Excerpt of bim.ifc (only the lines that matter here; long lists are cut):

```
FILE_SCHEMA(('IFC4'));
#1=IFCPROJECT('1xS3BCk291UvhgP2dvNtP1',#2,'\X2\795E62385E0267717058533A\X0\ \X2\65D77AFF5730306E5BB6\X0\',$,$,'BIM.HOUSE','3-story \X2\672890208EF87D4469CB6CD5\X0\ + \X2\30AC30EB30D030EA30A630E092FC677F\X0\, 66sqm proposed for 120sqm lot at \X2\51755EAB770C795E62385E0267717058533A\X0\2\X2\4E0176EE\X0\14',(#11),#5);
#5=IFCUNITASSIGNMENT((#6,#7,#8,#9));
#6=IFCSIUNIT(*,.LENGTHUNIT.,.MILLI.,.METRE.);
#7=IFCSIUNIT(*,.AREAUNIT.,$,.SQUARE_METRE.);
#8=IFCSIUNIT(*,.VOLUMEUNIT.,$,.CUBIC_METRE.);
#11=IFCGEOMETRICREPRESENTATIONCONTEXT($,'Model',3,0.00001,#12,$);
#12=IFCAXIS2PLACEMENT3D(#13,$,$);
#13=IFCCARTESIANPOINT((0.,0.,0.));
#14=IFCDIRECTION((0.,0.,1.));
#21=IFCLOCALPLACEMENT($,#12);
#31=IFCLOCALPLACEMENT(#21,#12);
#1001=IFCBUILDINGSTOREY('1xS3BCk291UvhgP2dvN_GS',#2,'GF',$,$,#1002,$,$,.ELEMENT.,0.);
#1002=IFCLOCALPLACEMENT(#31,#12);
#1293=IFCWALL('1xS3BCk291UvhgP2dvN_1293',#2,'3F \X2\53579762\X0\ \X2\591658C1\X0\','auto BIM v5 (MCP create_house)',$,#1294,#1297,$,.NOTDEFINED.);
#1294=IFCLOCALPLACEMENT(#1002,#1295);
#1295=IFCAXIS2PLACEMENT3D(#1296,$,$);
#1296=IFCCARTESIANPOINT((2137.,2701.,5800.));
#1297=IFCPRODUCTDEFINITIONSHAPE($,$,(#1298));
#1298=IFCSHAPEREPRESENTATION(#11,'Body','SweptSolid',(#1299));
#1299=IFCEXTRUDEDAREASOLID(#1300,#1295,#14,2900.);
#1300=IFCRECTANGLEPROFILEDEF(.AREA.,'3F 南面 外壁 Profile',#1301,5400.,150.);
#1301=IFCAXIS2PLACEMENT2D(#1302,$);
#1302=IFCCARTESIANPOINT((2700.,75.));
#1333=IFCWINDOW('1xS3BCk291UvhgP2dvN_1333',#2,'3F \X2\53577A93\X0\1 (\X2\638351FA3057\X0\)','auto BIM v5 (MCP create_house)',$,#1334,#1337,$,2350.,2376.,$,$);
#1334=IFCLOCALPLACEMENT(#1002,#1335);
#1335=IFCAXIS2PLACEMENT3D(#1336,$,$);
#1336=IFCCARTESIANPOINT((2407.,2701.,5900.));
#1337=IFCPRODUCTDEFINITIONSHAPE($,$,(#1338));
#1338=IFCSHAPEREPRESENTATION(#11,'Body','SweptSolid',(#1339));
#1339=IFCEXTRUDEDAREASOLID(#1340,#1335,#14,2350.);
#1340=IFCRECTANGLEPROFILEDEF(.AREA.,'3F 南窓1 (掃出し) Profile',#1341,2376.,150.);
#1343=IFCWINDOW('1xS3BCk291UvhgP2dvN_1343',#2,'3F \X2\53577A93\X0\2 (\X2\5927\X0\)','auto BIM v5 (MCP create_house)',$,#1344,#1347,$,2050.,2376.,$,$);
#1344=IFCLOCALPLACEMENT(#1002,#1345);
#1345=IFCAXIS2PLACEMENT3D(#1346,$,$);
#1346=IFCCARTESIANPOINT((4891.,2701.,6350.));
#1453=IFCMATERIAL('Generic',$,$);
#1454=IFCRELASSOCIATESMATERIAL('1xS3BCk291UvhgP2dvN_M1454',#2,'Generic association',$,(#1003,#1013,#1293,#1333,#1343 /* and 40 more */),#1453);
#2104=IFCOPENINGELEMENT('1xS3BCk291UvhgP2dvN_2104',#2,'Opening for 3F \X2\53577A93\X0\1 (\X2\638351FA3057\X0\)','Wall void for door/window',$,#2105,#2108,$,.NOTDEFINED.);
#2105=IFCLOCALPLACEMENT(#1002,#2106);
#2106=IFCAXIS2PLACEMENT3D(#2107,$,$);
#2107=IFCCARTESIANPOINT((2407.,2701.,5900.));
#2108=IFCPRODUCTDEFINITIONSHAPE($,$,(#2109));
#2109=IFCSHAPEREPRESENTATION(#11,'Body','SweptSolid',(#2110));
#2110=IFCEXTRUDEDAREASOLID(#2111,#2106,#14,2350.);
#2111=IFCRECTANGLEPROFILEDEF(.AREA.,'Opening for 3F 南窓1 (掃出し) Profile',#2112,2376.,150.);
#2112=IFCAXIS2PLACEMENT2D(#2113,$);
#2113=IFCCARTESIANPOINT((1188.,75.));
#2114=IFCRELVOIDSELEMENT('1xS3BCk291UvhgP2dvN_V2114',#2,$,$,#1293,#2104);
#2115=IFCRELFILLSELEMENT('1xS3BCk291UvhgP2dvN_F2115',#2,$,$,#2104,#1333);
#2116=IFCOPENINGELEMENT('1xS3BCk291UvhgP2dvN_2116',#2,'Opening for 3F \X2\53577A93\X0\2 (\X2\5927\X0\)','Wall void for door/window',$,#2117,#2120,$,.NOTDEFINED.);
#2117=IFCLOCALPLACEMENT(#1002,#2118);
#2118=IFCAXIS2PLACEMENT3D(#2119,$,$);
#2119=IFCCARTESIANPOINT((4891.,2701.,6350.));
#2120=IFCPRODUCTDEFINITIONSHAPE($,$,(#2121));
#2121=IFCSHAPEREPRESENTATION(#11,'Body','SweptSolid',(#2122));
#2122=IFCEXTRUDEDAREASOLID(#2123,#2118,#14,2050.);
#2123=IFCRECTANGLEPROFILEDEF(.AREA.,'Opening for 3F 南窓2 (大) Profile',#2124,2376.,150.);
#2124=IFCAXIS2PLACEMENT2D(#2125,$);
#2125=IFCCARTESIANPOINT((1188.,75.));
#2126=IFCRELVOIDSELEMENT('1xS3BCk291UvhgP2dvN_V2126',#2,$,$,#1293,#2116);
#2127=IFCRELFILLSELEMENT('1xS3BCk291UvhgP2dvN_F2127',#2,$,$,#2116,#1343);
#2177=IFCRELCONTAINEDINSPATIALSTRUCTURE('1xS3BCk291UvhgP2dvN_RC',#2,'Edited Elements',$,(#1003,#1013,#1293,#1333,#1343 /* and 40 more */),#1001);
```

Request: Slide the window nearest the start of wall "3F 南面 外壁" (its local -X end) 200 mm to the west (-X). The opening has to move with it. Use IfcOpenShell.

```python
import ifcopenshell
import ifcopenshell.api.geometry
import ifcopenshell.util.placement

model = ifcopenshell.open("bim.ifc")

window = model.by_id(1333)
opening = window.FillsVoids[0].RelatingOpeningElement
wall = opening.VoidsElements[0].RelatingBuildingElement

wall_matrix = ifcopenshell.util.placement.get_local_placement(wall.ObjectPlacement)
shift = wall_matrix[:3, 0] * -200.0
before = ifcopenshell.util.placement.get_local_placement(window.ObjectPlacement)[:3, 3].copy()

# The window is not placed relative to its opening, so move both.
for product in (opening, window):
    matrix = ifcopenshell.util.placement.get_local_placement(product.ObjectPlacement)
    matrix[:3, 3] += shift
    ifcopenshell.api.geometry.edit_object_placement(model, product=product, matrix=matrix, is_si=False)

after = ifcopenshell.util.placement.get_local_placement(window.ObjectPlacement)[:3, 3]
print("window moved by", (after - before).round(3) + 0.0)

model.write("bim_updated.ifc")
```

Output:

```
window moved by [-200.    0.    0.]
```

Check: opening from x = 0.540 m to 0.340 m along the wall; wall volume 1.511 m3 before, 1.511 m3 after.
